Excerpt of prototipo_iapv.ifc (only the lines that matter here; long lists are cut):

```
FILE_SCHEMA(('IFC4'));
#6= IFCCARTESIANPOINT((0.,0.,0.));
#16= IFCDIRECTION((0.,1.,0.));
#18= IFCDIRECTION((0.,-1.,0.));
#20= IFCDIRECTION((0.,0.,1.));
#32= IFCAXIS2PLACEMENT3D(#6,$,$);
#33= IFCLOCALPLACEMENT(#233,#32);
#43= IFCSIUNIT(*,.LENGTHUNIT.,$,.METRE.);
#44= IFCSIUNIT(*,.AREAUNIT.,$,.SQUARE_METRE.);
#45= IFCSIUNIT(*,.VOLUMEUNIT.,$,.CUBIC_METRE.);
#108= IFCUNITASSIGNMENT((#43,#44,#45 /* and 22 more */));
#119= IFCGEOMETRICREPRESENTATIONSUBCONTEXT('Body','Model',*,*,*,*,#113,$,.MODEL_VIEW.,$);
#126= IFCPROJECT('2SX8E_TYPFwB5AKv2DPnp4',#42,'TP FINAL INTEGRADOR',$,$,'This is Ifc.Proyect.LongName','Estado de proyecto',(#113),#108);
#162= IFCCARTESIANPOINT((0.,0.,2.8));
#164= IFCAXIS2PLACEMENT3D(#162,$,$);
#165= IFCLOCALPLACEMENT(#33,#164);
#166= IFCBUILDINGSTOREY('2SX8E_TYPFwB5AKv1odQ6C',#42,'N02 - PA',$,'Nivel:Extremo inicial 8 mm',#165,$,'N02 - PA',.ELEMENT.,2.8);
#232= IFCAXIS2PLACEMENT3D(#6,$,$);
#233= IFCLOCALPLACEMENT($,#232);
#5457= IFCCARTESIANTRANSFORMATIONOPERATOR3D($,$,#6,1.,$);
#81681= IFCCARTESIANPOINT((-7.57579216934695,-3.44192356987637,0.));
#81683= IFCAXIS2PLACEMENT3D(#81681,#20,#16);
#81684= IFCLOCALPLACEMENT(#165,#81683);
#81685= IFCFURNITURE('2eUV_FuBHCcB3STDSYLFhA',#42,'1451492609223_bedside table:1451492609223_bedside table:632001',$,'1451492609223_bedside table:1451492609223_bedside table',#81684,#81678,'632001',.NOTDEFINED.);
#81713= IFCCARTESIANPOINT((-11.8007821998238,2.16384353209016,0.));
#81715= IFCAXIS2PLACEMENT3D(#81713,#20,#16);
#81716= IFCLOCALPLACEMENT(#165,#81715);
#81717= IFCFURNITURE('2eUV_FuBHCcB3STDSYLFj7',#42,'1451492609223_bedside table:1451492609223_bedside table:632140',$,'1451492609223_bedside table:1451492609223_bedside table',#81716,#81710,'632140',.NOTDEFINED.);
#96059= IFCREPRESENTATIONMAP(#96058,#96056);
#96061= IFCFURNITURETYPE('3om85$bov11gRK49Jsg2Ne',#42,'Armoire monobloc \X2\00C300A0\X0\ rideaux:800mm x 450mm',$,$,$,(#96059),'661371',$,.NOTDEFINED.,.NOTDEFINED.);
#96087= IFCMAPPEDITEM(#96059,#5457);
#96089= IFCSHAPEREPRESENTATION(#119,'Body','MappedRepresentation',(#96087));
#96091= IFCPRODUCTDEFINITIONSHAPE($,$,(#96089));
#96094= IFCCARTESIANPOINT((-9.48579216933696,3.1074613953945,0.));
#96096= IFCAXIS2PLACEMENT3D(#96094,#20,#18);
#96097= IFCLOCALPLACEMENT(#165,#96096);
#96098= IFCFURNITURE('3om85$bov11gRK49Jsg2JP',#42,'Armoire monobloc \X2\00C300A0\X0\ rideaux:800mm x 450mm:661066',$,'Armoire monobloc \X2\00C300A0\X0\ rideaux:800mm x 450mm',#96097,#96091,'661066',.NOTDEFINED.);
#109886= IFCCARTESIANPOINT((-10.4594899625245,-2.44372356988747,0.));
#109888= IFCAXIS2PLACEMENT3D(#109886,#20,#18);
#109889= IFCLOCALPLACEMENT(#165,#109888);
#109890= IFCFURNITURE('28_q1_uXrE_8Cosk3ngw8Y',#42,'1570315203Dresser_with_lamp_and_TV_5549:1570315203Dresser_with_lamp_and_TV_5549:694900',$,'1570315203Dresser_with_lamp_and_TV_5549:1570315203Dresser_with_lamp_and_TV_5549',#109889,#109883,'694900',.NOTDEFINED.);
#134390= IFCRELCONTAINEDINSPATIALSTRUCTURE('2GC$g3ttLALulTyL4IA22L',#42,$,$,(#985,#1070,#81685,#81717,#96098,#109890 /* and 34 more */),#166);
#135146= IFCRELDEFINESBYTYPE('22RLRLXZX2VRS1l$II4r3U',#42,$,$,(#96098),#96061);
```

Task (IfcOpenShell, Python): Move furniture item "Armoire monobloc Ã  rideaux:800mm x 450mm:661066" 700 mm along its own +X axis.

```python
import ifcopenshell
import ifcopenshell.api.geometry
import ifcopenshell.util.placement
import ifcopenshell.util.unit

model = ifcopenshell.open("prototipo_iapv.ifc")
unit_scale = ifcopenshell.util.unit.calculate_unit_scale(model)

item = model.by_id(96098)
matrix = ifcopenshell.util.placement.get_local_placement(item.ObjectPlacement)
matrix[:3, 3] += matrix[:3, 0] * 0.7 / unit_scale
ifcopenshell.api.geometry.edit_object_placement(model, product=item, matrix=matrix, is_si=False)

print(ifcopenshell.util.placement.get_local_placement(item.ObjectPlacement).round(3) + 0.0)

model.write("prototipo_iapv-out.ifc")
```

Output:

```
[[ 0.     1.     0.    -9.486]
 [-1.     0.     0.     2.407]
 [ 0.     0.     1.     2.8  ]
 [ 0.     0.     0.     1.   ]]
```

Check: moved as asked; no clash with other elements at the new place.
